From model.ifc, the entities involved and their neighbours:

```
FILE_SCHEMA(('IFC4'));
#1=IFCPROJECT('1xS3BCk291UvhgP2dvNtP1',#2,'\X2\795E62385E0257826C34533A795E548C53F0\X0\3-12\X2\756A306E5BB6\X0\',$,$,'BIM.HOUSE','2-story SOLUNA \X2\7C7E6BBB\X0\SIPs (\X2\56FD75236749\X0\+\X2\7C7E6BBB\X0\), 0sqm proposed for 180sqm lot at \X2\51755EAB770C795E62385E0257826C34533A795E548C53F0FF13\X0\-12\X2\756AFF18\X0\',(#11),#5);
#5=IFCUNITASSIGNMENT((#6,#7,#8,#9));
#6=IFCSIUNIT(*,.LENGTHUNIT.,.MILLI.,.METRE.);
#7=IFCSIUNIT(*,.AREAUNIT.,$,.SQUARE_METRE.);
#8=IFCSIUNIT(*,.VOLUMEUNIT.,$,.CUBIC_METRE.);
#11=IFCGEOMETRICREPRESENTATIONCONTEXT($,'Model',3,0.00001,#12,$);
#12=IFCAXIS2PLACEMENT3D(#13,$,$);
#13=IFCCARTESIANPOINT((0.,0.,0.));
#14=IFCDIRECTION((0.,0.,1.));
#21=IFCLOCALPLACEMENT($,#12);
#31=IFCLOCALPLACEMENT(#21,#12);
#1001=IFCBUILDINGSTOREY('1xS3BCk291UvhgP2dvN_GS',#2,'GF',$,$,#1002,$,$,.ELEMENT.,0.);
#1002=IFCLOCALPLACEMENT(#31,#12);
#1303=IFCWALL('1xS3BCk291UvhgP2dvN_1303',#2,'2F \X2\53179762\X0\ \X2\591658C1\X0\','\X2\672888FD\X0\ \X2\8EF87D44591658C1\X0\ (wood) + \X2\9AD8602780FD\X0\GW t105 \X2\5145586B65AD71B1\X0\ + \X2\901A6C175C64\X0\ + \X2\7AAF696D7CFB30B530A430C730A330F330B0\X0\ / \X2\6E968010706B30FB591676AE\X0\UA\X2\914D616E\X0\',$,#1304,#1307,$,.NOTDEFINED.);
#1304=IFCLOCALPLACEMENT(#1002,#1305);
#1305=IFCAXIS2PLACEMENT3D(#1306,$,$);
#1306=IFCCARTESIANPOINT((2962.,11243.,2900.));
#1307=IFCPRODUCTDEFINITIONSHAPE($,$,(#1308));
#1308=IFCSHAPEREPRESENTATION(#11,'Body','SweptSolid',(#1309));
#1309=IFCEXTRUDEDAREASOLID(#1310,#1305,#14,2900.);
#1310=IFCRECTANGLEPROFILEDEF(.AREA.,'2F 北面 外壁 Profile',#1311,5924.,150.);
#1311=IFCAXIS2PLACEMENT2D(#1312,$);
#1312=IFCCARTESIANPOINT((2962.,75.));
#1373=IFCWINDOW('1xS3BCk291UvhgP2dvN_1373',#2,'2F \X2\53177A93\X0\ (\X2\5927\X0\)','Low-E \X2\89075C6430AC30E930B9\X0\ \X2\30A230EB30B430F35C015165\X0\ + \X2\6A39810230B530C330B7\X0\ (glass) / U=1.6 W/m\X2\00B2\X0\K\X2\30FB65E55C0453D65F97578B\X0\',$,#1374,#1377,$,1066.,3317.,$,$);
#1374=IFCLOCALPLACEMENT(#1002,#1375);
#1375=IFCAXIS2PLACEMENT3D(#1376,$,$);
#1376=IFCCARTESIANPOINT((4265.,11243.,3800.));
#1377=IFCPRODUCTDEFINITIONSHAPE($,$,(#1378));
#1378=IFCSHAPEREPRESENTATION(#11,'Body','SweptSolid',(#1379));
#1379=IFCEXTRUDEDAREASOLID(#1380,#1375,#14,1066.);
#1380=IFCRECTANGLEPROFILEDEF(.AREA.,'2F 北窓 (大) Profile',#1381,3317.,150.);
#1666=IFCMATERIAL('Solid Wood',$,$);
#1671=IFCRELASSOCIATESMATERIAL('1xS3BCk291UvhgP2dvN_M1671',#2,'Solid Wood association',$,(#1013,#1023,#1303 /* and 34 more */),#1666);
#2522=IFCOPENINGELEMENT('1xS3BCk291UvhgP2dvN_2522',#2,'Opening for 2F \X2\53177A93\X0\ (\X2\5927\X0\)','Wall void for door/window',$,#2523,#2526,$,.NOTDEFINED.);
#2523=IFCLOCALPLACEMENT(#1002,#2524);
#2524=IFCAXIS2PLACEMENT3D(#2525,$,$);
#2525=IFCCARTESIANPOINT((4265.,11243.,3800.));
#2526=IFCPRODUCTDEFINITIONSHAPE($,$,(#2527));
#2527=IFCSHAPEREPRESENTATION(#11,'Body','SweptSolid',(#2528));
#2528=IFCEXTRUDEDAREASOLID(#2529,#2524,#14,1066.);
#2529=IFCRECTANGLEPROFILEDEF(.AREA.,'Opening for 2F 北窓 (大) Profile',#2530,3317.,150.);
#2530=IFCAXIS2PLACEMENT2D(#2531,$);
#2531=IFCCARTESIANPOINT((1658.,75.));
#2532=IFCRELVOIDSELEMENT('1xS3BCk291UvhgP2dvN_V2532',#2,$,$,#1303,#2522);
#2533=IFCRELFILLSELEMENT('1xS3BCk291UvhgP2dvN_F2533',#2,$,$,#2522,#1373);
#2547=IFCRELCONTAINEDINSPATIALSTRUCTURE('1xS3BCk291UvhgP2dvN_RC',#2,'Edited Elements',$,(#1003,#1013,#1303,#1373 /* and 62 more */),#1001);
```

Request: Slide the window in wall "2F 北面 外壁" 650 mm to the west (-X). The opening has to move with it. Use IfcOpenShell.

```python
import ifcopenshell
import ifcopenshell.api.geometry
import ifcopenshell.util.placement

model = ifcopenshell.open("model.ifc")

window = model.by_id(1373)
opening = window.FillsVoids[0].RelatingOpeningElement
wall = opening.VoidsElements[0].RelatingBuildingElement

wall_matrix = ifcopenshell.util.placement.get_local_placement(wall.ObjectPlacement)
shift = wall_matrix[:3, 0] * -650.0
before = ifcopenshell.util.placement.get_local_placement(window.ObjectPlacement)[:3, 3].copy()

# The window is not placed relative to its opening, so move both.
for product in (opening, window):
    matrix = ifcopenshell.util.placement.get_local_placement(product.ObjectPlacement)
    matrix[:3, 3] += shift
    ifcopenshell.api.geometry.edit_object_placement(model, product=product, matrix=matrix, is_si=False)

after = ifcopenshell.util.placement.get_local_placement(window.ObjectPlacement)[:3, 3]
print("window moved by", (after - before).round(3) + 0.0)

model.write("model_v2.ifc")
```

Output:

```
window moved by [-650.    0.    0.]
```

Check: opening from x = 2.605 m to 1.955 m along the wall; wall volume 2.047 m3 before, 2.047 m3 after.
